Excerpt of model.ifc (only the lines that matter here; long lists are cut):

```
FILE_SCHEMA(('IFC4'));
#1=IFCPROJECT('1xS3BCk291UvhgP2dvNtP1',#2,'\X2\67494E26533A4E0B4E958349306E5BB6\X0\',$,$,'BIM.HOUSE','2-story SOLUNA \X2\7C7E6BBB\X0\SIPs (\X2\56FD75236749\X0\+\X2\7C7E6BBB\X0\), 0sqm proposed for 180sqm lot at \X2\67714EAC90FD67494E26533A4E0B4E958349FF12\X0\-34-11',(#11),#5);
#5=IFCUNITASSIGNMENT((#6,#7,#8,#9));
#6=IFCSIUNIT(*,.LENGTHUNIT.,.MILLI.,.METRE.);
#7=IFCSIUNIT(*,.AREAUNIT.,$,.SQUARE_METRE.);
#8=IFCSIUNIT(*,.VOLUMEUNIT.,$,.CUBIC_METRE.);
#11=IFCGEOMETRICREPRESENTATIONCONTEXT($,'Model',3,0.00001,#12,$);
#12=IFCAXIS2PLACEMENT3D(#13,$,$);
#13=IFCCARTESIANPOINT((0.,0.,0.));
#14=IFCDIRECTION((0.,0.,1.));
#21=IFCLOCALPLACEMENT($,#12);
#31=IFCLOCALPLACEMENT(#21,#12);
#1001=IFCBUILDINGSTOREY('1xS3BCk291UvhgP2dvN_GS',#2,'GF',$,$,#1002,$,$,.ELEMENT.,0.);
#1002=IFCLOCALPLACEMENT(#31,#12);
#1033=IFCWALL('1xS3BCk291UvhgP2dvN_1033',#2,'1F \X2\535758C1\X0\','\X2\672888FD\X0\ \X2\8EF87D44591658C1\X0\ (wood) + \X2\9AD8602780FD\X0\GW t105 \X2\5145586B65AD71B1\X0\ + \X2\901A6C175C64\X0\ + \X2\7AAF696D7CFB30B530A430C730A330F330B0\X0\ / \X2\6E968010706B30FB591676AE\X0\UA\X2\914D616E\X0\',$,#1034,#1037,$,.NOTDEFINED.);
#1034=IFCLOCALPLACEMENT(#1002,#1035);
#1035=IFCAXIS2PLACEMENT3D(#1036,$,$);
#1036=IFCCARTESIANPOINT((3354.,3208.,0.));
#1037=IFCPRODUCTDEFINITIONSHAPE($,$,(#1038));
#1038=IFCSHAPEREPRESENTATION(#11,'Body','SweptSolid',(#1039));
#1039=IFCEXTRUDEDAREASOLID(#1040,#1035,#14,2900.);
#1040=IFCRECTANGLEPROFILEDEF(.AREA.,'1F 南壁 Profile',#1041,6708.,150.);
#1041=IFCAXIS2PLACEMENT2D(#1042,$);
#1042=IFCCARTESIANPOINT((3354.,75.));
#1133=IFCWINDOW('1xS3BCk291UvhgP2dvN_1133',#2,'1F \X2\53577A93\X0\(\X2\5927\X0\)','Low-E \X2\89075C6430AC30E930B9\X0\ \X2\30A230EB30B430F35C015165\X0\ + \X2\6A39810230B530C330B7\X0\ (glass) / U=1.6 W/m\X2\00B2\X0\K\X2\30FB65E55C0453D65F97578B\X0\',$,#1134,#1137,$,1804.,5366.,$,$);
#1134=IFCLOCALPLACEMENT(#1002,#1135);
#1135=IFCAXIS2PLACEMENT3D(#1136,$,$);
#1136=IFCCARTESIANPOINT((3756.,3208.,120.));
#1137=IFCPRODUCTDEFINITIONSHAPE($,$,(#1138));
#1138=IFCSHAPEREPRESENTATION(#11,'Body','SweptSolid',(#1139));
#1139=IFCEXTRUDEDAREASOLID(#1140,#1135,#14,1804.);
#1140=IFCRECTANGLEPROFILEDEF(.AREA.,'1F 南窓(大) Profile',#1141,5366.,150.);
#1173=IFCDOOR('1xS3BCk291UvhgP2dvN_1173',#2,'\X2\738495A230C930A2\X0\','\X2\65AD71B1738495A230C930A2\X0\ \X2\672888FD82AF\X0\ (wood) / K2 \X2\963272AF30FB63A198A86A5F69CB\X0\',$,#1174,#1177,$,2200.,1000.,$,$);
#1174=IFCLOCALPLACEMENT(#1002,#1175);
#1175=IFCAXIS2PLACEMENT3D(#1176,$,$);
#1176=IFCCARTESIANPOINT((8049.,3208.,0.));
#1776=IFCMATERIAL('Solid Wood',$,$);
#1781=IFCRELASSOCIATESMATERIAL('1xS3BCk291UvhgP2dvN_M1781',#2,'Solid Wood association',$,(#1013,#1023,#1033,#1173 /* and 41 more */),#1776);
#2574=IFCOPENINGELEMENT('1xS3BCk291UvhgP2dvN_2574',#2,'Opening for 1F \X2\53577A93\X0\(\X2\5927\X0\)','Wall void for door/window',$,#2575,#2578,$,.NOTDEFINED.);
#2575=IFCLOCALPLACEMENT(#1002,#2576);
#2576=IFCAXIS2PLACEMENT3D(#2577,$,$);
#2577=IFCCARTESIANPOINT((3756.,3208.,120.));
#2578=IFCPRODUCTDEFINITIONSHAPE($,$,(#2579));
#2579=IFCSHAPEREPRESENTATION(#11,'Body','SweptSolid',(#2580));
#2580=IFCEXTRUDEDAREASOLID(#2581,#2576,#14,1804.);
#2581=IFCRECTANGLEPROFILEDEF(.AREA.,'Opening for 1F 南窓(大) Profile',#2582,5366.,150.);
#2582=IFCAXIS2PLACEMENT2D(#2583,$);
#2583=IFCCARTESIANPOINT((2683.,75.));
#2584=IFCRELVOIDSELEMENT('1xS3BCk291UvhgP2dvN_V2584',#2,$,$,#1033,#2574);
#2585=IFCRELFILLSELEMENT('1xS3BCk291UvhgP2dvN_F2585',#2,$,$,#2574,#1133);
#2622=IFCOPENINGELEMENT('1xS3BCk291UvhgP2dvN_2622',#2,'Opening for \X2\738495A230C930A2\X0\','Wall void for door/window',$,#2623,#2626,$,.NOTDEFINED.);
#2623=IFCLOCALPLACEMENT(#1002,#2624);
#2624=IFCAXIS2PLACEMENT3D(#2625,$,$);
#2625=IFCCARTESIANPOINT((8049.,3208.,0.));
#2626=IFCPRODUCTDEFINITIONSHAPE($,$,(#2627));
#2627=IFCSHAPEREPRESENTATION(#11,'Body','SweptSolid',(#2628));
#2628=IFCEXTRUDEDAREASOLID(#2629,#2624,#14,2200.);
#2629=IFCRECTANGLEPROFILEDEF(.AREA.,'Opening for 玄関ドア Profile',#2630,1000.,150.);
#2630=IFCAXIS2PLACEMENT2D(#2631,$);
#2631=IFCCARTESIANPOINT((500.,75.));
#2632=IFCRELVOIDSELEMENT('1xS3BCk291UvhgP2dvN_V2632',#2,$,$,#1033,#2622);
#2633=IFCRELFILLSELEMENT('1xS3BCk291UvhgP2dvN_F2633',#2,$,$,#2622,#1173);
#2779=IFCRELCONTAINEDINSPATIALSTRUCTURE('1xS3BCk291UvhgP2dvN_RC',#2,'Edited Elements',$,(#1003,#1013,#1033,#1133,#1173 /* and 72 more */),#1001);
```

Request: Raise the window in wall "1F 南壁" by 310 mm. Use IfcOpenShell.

```python
import numpy as np
import ifcopenshell
import ifcopenshell.api.geometry
import ifcopenshell.util.placement
import ifcopenshell.util.unit

model = ifcopenshell.open("model.ifc")
unit_scale = ifcopenshell.util.unit.calculate_unit_scale(model)

window = model.by_guid("1xS3BCk291UvhgP2dvN_1133")
opening = window.FillsVoids[0].RelatingOpeningElement
dz = 0.31 / unit_scale

shift = np.array([0.0, 0.0, dz])
# The window is not placed relative to its opening, so move both.
for product in (opening, window):
    matrix = ifcopenshell.util.placement.get_local_placement(product.ObjectPlacement)
    matrix[:3, 3] += shift
    ifcopenshell.api.geometry.edit_object_placement(model, product=product, matrix=matrix, is_si=False)

print(f"moved by {dz * unit_scale:+.3f} m")

model.write("model-out.ifc")
```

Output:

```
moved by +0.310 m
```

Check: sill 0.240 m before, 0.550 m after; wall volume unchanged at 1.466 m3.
